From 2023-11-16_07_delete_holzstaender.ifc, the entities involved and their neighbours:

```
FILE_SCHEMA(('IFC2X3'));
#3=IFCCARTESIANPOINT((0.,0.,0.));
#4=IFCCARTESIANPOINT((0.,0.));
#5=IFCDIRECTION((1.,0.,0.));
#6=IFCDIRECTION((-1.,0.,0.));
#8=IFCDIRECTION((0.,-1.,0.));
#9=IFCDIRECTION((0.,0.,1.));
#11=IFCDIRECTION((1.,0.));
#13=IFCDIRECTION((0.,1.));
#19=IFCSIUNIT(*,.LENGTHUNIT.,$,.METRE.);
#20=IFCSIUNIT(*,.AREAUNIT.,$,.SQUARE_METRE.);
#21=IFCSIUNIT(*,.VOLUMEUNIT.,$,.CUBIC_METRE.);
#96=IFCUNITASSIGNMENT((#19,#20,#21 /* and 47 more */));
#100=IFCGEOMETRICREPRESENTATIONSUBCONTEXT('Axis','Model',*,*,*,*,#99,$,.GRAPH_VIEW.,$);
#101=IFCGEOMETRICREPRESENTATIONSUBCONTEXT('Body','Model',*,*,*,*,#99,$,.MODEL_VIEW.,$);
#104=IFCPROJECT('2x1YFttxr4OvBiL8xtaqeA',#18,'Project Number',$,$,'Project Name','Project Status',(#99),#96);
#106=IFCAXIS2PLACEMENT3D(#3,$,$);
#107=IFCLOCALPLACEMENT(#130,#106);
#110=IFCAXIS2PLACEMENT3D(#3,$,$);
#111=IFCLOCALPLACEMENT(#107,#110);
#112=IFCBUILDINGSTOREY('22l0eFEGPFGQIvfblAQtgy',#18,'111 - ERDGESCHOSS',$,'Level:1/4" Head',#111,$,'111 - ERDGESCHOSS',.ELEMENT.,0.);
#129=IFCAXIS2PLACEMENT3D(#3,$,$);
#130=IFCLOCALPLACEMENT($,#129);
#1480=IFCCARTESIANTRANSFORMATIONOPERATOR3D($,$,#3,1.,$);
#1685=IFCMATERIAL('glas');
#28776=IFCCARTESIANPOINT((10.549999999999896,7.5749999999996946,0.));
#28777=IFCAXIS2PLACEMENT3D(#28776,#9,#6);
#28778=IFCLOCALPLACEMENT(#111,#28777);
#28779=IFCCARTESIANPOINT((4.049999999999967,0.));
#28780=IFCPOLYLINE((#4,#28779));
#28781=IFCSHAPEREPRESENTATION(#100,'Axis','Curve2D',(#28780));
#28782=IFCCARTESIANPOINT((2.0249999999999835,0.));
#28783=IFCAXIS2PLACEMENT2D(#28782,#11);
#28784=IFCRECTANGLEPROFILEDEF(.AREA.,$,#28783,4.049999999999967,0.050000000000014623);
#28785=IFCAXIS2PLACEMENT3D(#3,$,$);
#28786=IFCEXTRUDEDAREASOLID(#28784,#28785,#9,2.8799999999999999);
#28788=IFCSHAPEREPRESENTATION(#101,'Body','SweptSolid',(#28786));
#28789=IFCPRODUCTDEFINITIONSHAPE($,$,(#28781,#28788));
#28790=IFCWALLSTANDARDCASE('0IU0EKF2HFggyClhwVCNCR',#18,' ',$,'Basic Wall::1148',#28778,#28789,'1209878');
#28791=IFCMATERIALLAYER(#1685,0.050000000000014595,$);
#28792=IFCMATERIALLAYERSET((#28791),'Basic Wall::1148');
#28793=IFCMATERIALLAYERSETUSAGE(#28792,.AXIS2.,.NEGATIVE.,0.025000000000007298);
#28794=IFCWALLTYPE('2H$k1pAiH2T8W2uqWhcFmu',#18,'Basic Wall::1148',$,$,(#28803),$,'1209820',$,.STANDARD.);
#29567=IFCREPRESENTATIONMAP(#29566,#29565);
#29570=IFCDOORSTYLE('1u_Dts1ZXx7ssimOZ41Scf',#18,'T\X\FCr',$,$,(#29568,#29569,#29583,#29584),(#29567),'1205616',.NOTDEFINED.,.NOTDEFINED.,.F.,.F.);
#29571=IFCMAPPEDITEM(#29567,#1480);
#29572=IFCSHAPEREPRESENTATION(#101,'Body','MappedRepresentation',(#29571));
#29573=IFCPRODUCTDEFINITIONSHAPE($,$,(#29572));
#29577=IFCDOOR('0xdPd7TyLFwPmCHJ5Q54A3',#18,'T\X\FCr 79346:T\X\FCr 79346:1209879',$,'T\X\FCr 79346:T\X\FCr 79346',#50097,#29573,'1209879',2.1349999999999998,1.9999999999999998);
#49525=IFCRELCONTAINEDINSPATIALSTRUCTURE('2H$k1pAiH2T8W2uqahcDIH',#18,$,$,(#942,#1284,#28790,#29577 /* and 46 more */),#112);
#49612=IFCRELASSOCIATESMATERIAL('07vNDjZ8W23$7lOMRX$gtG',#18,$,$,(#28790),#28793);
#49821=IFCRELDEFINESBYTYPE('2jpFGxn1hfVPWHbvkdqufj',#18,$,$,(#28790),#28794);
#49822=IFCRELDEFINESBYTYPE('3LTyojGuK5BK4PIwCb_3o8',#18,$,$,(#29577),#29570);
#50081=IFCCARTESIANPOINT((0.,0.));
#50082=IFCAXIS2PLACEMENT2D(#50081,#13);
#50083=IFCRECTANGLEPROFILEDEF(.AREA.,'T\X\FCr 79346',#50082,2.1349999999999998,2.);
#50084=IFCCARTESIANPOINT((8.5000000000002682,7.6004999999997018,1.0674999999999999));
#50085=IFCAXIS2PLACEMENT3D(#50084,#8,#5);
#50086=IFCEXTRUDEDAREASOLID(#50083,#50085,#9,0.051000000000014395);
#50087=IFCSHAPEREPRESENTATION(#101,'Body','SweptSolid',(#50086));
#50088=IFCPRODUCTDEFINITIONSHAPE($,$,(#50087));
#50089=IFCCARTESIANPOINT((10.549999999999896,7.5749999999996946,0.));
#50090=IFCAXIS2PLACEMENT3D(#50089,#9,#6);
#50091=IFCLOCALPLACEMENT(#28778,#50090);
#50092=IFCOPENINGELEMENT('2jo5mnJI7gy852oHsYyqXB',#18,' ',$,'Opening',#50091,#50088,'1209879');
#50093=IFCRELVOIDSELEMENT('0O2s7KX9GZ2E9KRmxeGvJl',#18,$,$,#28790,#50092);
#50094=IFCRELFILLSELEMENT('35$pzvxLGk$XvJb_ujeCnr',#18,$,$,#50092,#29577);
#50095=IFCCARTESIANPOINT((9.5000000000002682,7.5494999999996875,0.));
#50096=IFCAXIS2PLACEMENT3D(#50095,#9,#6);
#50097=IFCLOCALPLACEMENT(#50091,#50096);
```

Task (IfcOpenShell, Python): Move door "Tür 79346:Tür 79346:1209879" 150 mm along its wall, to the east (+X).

```python
import ifcopenshell
import ifcopenshell.api.geometry
import ifcopenshell.util.placement
import ifcopenshell.util.unit

model = ifcopenshell.open("2023-11-16_07_delete_holzstaender.ifc")
unit_scale = ifcopenshell.util.unit.calculate_unit_scale(model)

door = model.by_guid("0xdPd7TyLFwPmCHJ5Q54A3")
opening = door.FillsVoids[0].RelatingOpeningElement
wall = opening.VoidsElements[0].RelatingBuildingElement

wall_matrix = ifcopenshell.util.placement.get_local_placement(wall.ObjectPlacement)
shift = wall_matrix[:3, 0] * -0.15 / unit_scale
before = ifcopenshell.util.placement.get_local_placement(door.ObjectPlacement)[:3, 3].copy()

# The door is placed relative to its opening, so it follows when the opening moves.
matrix = ifcopenshell.util.placement.get_local_placement(opening.ObjectPlacement)
matrix[:3, 3] += shift
ifcopenshell.api.geometry.edit_object_placement(
    model, product=opening, matrix=matrix, is_si=False, should_transform_children=True
)

after = ifcopenshell.util.placement.get_local_placement(door.ObjectPlacement)[:3, 3]
print("door moved by", (after - before).round(3) + 0.0)

model.write("2023-11-16_07_delete_holzstaender_v2.ifc")
```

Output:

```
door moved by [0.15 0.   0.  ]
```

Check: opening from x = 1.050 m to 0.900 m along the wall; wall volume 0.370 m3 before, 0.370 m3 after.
